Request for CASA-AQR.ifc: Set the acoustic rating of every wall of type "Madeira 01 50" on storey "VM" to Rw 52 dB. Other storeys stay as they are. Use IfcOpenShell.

First a look at what the model holds.

```python
import ifcopenshell
import ifcopenshell.util.element

model = ifcopenshell.open("CASA-AQR.ifc")
print(model.schema)
storey = next(s for s in model.by_type("IfcBuildingStorey") if s.Name == "VM")
walls = [e for e in ifcopenshell.util.element.get_decomposition(storey) if e.is_a("IfcWall")]
seen = {}
for e in walls:
    element_type = ifcopenshell.util.element.get_type(e)
    key = (element_type.Name if element_type != e and element_type else None, ifcopenshell.util.element.get_pset(e, "Pset_WallCommon", "AcousticRating"))
    seen[key] = seen.get(key, 0) + 1
for (name, value), count in sorted(seen.items(), key=str):
    print(count, "x", name, "|", value)
```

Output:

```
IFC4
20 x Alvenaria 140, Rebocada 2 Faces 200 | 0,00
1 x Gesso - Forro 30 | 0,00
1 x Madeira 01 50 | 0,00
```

```python
import ifcopenshell
import ifcopenshell.api.pset
import ifcopenshell.util.element

model = ifcopenshell.open("CASA-AQR.ifc")

storey = next(s for s in model.by_type("IfcBuildingStorey") if s.Name == "VM")
walls = [e for e in ifcopenshell.util.element.get_decomposition(storey) if e.is_a("IfcWall")]

count = 0
for e in walls:
    element_type = ifcopenshell.util.element.get_type(e)
    if element_type in (None, e) or element_type.Name != "Madeira 01 50":
        continue
    # add_pset returns the element's existing set when there is one.
    pset = ifcopenshell.api.pset.add_pset(model, product=e, name="Pset_WallCommon")
    ifcopenshell.api.pset.edit_pset(model, pset=pset, properties={"AcousticRating": "Rw 52 dB"})
    count += 1

print(count, "walls updated")

model.write("CASA-AQR_updated.ifc")
```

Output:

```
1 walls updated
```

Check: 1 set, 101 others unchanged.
